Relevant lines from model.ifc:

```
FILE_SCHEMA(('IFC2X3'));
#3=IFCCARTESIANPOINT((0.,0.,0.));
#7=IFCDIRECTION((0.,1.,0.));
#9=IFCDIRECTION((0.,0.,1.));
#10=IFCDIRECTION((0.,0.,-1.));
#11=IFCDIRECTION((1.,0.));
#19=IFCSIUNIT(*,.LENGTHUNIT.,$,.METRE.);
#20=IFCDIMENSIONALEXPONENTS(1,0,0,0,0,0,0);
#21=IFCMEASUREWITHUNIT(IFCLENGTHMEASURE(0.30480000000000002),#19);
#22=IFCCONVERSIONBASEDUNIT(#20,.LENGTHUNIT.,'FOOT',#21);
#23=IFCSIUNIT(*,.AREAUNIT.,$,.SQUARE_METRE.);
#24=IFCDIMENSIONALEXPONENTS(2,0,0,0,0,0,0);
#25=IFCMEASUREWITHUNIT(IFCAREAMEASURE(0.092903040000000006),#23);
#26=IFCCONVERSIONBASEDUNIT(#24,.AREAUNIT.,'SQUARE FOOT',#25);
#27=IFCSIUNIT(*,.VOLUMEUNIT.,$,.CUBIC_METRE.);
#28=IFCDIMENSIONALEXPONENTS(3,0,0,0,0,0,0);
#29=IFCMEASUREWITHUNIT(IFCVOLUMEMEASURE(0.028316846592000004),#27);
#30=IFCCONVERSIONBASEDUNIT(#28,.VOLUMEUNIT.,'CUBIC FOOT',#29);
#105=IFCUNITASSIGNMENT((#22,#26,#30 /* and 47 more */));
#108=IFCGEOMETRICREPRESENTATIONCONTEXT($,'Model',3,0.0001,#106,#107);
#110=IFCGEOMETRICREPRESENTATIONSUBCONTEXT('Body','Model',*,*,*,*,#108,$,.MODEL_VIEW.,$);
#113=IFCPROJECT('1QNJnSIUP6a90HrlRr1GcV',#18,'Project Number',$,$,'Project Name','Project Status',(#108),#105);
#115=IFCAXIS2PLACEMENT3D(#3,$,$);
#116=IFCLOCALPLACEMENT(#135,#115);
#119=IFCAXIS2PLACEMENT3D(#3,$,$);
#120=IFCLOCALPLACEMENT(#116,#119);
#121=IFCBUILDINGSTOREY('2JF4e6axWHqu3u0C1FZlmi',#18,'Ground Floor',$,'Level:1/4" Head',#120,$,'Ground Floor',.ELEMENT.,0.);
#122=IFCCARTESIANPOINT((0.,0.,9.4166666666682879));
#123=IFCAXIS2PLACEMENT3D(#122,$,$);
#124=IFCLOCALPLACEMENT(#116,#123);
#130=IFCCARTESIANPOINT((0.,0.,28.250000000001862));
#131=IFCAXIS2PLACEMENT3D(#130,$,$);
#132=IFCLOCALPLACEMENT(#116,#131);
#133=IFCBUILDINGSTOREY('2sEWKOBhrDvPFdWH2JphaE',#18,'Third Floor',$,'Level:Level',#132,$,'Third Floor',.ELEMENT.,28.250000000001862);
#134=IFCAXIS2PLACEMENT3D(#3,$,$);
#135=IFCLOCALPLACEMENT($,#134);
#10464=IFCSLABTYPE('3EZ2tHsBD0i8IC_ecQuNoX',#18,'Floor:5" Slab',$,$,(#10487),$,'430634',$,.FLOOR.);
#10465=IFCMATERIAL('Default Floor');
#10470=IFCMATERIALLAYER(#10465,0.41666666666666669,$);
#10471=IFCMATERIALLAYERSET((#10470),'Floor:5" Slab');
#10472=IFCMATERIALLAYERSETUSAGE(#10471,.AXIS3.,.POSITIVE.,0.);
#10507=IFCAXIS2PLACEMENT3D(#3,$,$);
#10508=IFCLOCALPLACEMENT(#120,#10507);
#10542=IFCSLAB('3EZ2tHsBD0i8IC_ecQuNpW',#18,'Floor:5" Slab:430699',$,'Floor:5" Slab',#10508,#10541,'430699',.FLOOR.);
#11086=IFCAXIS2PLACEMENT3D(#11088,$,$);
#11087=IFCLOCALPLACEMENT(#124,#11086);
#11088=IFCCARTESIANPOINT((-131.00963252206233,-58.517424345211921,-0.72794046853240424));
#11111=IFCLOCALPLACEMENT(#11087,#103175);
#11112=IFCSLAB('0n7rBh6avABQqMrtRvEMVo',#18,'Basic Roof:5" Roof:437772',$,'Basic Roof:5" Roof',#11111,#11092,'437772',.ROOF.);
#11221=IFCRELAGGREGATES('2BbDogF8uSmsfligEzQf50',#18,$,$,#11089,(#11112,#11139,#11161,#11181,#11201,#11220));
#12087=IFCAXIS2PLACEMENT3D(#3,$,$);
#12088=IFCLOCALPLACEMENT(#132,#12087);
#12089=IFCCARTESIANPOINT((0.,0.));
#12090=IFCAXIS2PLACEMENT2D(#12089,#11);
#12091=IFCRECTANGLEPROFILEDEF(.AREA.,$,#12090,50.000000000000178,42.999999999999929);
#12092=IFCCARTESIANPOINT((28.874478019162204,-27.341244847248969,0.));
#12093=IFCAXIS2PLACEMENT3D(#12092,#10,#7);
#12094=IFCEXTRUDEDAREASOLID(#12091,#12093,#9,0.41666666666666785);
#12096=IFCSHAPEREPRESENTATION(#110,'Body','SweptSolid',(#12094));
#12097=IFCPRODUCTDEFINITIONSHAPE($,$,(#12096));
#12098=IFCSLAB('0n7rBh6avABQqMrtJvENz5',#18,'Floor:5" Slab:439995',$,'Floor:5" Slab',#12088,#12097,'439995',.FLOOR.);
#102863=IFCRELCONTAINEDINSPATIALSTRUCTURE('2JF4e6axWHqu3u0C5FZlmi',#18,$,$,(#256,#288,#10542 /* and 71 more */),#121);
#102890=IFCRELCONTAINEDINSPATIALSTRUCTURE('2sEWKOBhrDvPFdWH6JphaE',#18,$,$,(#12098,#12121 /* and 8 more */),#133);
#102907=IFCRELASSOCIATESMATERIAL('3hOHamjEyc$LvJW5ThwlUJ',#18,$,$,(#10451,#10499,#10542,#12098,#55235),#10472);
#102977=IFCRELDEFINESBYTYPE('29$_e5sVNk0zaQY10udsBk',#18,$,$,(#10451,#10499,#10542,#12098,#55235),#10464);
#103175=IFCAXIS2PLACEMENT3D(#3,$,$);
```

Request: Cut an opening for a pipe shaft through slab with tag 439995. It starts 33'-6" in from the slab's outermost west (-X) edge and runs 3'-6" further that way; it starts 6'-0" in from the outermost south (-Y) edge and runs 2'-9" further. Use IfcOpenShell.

```python
import numpy as np
import ifcopenshell
import ifcopenshell.api.feature
import ifcopenshell.api.geometry
import ifcopenshell.api.root
import ifcopenshell.geom
import ifcopenshell.util.placement
import ifcopenshell.util.representation
import ifcopenshell.util.shape
import ifcopenshell.util.unit

model = ifcopenshell.open("model.ifc")
unit_scale = ifcopenshell.util.unit.calculate_unit_scale(model)
settings = ifcopenshell.geom.settings()


def volume(element):
    """Net volume in cubic metres, openings subtracted."""
    shape = ifcopenshell.geom.create_shape(settings, element)
    return ifcopenshell.util.shape.get_volume(shape.geometry)


slab = model.by_guid("0n7rBh6avABQqMrtJvENz5")
before = volume(slab)

# Extent in the slab's own axes, in metres. The edges named are its -X and -Y sides.
slab_shape = ifcopenshell.geom.create_shape(settings, slab)
vertices = ifcopenshell.util.shape.get_vertices(slab_shape.geometry)
x_min, y_min, bottom = vertices.min(axis=0)
top = vertices[:, 2].max()

opening = ifcopenshell.api.root.create_entity(model, ifc_class="IfcOpeningElement", name="Pipe shaft opening")
context = ifcopenshell.util.representation.get_context(model, "Model", "Body", "MODEL_VIEW")
width, depth = 1.0668, 0.8382
outline = [(0.0, 0.0), (width, 0.0), (width, depth), (0.0, depth), (0.0, 0.0)]
# Overshoot both faces by 50 mm so the cut is clean.
shape = ifcopenshell.api.geometry.add_slab_representation(
    model, context=context, depth=top - bottom + 0.1, polyline=outline
)
ifcopenshell.api.geometry.assign_representation(model, product=opening, representation=shape)

matrix = ifcopenshell.util.placement.get_local_placement(slab.ObjectPlacement)
matrix[:, 3] = matrix @ np.append(np.array([x_min + 10.2108, y_min + 1.8288, bottom - 0.05]) / unit_scale, 1.0)
ifcopenshell.api.geometry.edit_object_placement(model, product=opening, matrix=matrix, is_si=False)
ifcopenshell.api.feature.add_feature(model, feature=opening, element=slab)

after = volume(slab)

print(f"slab volume {before:.3f} -> {after:.3f} m3")

model.write("model-out.ifc")
```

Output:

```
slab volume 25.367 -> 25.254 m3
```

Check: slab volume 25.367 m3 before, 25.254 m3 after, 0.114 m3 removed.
